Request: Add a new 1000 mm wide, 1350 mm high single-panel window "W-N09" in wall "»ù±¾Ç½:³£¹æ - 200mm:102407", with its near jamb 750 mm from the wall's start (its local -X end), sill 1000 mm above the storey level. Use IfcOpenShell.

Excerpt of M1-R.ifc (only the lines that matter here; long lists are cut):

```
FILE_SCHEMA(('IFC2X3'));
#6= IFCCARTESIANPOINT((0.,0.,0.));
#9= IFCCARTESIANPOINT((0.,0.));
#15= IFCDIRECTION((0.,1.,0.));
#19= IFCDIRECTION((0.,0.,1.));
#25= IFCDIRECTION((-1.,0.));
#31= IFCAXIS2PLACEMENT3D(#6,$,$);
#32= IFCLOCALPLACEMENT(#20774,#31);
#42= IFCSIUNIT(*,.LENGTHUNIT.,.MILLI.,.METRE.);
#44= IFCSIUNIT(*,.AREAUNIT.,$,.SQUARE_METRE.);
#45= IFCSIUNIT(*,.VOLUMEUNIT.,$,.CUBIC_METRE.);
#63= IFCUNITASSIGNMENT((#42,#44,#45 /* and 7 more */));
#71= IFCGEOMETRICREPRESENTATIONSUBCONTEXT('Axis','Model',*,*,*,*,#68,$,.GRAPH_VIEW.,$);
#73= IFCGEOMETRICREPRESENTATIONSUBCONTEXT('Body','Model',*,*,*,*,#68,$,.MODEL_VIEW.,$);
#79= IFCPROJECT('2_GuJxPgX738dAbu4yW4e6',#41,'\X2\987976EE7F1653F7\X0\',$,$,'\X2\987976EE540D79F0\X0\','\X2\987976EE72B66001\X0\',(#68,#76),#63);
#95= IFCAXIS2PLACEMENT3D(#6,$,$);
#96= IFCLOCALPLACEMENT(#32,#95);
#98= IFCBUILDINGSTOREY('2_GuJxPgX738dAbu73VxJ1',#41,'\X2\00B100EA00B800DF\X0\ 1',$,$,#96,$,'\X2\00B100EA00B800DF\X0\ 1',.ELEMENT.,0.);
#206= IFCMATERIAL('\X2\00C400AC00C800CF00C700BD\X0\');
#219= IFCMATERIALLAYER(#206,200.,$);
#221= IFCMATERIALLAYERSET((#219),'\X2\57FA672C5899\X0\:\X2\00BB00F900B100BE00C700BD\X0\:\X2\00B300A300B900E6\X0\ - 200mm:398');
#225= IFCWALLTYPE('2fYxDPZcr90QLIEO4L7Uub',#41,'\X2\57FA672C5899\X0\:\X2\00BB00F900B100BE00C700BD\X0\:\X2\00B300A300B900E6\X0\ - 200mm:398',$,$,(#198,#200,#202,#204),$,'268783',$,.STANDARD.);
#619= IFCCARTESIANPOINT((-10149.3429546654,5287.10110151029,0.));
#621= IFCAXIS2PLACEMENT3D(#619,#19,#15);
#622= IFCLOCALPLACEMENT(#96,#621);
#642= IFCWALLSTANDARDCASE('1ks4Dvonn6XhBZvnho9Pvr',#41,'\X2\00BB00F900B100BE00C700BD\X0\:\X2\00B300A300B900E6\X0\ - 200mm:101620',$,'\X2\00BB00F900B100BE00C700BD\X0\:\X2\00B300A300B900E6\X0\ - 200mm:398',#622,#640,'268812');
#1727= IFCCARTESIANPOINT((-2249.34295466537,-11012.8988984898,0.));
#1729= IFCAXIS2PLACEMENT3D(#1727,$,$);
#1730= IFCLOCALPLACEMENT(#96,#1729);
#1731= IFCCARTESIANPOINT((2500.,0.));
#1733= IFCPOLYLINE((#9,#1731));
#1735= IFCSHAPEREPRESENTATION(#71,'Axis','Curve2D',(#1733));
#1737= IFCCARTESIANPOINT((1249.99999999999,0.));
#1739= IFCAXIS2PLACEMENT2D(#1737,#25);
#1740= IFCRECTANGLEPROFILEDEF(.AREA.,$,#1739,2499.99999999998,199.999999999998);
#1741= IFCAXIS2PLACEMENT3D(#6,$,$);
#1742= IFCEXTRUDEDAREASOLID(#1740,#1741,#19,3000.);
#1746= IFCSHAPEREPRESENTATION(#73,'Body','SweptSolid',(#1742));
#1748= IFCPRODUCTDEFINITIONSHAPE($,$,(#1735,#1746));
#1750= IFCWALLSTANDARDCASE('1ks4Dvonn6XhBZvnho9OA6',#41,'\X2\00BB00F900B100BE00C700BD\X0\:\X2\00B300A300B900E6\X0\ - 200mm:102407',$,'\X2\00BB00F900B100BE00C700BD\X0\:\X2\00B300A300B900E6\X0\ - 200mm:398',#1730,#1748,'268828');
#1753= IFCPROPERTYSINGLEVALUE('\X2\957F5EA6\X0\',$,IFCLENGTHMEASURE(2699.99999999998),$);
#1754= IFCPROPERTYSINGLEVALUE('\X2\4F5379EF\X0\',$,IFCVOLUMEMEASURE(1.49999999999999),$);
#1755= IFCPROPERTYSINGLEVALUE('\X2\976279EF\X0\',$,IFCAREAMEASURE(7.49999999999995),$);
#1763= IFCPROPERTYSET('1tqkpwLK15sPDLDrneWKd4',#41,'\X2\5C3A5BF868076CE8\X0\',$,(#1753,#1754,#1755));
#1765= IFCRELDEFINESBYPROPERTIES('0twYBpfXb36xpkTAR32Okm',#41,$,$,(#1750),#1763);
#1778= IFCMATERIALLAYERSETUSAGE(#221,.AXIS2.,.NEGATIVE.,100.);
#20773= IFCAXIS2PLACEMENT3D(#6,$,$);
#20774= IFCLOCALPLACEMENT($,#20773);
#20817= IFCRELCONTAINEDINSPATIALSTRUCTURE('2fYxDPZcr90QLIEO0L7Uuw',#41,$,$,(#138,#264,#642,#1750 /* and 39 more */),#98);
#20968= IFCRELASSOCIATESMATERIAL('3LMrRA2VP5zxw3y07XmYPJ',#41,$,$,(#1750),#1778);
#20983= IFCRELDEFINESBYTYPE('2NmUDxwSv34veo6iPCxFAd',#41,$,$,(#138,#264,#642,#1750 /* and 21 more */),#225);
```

```python
import numpy as np
import ifcopenshell
import ifcopenshell.api.feature
import ifcopenshell.api.geometry
import ifcopenshell.api.pset
import ifcopenshell.api.root
import ifcopenshell.api.spatial
import ifcopenshell.api.type
import ifcopenshell.geom
import ifcopenshell.util.element
import ifcopenshell.util.placement
import ifcopenshell.util.representation
import ifcopenshell.util.shape
import ifcopenshell.util.unit

model = ifcopenshell.open("M1-R.ifc")
unit_scale = ifcopenshell.util.unit.calculate_unit_scale(model)
area_scale = ifcopenshell.util.unit.calculate_unit_scale(model, "AREAUNIT")
volume_scale = ifcopenshell.util.unit.calculate_unit_scale(model, "VOLUMEUNIT")
settings = ifcopenshell.geom.settings()


def volume(element):
    """Net volume in cubic metres, openings subtracted."""
    shape = ifcopenshell.geom.create_shape(settings, element)
    return ifcopenshell.util.shape.get_volume(shape.geometry)


wall = model.by_guid("1ks4Dvonn6XhBZvnho9OA6")
storey = ifcopenshell.util.element.get_container(wall, ifc_class="IfcBuildingStorey")
context = ifcopenshell.util.representation.get_context(model, "Model", "Body", "MODEL_VIEW")
before = volume(wall)

width, height, from_end, sill = 1, 1.35, 0.75, 1  # metres

# The wall runs along its own X axis, and the end named is its -X end.
wall_shape = ifcopenshell.geom.create_shape(settings, wall)
x, y, z = ifcopenshell.util.shape.get_vertices(wall_shape.geometry).T
start = x.min() + from_end
face, thickness = float(y.min()), float(y.max() - y.min())
wall_matrix = ifcopenshell.util.placement.get_local_placement(wall.ObjectPlacement)
level = ifcopenshell.util.placement.get_local_placement(storey.ObjectPlacement)[2, 3]


def in_wall(x, y):
    """Placement at x, y metres in the wall's axes, at sill height."""
    matrix = wall_matrix.copy()
    matrix[:, 3] = wall_matrix @ np.array([x / unit_scale, y / unit_scale, 0.0, 1.0])
    matrix[2, 3] = level + sill / unit_scale
    return matrix


# Opening: a box that overshoots both wall faces by 50 mm.
opening = ifcopenshell.api.root.create_entity(model, ifc_class="IfcOpeningElement")
box = ifcopenshell.api.geometry.add_wall_representation(
    model, context=context, length=width, height=height, thickness=thickness + 0.1
)
ifcopenshell.api.geometry.assign_representation(model, product=opening, representation=box)
ifcopenshell.api.geometry.edit_object_placement(model, product=opening, matrix=in_wall(start, face - 0.05), is_si=False)
ifcopenshell.api.feature.add_feature(model, feature=opening, element=wall)

window = ifcopenshell.api.root.create_entity(model, ifc_class="IfcWindow", name="W-N09")
window.OverallWidth, window.OverallHeight = width / unit_scale, height / unit_scale
body = ifcopenshell.api.geometry.add_window_representation(
    model,
    context=context,
    overall_width=window.OverallWidth,
    overall_height=window.OverallHeight,
    partition_type="SINGLE_PANEL",
)
ifcopenshell.api.geometry.assign_representation(model, product=window, representation=body)
ifcopenshell.api.spatial.assign_container(model, products=[window], relating_structure=storey)
fills = ifcopenshell.api.feature.add_filling(model, opening=opening, element=window)
fills.OwnerHistory = window.OwnerHistory  # required in IFC2X3

# IFC2X3 keeps the operation on the window style.
style = ifcopenshell.api.root.create_entity(model, ifc_class="IfcWindowStyle", name="W-N09")
style.OperationType, style.ConstructionType = "SINGLE_PANEL", "NOTDEFINED"
style.ParameterTakesPrecedence = style.Sizeable = False
ifcopenshell.api.type.assign_type(model, related_objects=[window], relating_type=style)

# Centre the window in the wall's thickness.
ifcopenshell.api.geometry.edit_object_placement(model, product=window, matrix=in_wall(start, face), is_si=False)
window_shape = ifcopenshell.geom.create_shape(settings, window)
depth = ifcopenshell.util.shape.get_vertices(window_shape.geometry)[:, 1]
offset = face + thickness / 2 - (depth.min() + depth.max()) / 2
ifcopenshell.api.geometry.edit_object_placement(model, product=window, matrix=in_wall(start, offset), is_si=False)

after = volume(wall)

# Update the wall's stored quantities.
pset = model.by_id(ifcopenshell.util.element.get_pset(wall, "尺寸标注", should_inherit=False)["id"])
ifcopenshell.api.pset.edit_pset(model, pset=pset, properties={
    "体积": model.create_entity("IfcVolumeMeasure", after / volume_scale),
    "面积": model.create_entity("IfcAreaMeasure", after / thickness / area_scale),
})

print(f"wall volume {before:.3f} -> {after:.3f} m3")

model.write("M1-R_updated.ifc")
```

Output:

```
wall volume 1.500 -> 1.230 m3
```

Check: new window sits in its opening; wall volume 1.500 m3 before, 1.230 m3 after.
